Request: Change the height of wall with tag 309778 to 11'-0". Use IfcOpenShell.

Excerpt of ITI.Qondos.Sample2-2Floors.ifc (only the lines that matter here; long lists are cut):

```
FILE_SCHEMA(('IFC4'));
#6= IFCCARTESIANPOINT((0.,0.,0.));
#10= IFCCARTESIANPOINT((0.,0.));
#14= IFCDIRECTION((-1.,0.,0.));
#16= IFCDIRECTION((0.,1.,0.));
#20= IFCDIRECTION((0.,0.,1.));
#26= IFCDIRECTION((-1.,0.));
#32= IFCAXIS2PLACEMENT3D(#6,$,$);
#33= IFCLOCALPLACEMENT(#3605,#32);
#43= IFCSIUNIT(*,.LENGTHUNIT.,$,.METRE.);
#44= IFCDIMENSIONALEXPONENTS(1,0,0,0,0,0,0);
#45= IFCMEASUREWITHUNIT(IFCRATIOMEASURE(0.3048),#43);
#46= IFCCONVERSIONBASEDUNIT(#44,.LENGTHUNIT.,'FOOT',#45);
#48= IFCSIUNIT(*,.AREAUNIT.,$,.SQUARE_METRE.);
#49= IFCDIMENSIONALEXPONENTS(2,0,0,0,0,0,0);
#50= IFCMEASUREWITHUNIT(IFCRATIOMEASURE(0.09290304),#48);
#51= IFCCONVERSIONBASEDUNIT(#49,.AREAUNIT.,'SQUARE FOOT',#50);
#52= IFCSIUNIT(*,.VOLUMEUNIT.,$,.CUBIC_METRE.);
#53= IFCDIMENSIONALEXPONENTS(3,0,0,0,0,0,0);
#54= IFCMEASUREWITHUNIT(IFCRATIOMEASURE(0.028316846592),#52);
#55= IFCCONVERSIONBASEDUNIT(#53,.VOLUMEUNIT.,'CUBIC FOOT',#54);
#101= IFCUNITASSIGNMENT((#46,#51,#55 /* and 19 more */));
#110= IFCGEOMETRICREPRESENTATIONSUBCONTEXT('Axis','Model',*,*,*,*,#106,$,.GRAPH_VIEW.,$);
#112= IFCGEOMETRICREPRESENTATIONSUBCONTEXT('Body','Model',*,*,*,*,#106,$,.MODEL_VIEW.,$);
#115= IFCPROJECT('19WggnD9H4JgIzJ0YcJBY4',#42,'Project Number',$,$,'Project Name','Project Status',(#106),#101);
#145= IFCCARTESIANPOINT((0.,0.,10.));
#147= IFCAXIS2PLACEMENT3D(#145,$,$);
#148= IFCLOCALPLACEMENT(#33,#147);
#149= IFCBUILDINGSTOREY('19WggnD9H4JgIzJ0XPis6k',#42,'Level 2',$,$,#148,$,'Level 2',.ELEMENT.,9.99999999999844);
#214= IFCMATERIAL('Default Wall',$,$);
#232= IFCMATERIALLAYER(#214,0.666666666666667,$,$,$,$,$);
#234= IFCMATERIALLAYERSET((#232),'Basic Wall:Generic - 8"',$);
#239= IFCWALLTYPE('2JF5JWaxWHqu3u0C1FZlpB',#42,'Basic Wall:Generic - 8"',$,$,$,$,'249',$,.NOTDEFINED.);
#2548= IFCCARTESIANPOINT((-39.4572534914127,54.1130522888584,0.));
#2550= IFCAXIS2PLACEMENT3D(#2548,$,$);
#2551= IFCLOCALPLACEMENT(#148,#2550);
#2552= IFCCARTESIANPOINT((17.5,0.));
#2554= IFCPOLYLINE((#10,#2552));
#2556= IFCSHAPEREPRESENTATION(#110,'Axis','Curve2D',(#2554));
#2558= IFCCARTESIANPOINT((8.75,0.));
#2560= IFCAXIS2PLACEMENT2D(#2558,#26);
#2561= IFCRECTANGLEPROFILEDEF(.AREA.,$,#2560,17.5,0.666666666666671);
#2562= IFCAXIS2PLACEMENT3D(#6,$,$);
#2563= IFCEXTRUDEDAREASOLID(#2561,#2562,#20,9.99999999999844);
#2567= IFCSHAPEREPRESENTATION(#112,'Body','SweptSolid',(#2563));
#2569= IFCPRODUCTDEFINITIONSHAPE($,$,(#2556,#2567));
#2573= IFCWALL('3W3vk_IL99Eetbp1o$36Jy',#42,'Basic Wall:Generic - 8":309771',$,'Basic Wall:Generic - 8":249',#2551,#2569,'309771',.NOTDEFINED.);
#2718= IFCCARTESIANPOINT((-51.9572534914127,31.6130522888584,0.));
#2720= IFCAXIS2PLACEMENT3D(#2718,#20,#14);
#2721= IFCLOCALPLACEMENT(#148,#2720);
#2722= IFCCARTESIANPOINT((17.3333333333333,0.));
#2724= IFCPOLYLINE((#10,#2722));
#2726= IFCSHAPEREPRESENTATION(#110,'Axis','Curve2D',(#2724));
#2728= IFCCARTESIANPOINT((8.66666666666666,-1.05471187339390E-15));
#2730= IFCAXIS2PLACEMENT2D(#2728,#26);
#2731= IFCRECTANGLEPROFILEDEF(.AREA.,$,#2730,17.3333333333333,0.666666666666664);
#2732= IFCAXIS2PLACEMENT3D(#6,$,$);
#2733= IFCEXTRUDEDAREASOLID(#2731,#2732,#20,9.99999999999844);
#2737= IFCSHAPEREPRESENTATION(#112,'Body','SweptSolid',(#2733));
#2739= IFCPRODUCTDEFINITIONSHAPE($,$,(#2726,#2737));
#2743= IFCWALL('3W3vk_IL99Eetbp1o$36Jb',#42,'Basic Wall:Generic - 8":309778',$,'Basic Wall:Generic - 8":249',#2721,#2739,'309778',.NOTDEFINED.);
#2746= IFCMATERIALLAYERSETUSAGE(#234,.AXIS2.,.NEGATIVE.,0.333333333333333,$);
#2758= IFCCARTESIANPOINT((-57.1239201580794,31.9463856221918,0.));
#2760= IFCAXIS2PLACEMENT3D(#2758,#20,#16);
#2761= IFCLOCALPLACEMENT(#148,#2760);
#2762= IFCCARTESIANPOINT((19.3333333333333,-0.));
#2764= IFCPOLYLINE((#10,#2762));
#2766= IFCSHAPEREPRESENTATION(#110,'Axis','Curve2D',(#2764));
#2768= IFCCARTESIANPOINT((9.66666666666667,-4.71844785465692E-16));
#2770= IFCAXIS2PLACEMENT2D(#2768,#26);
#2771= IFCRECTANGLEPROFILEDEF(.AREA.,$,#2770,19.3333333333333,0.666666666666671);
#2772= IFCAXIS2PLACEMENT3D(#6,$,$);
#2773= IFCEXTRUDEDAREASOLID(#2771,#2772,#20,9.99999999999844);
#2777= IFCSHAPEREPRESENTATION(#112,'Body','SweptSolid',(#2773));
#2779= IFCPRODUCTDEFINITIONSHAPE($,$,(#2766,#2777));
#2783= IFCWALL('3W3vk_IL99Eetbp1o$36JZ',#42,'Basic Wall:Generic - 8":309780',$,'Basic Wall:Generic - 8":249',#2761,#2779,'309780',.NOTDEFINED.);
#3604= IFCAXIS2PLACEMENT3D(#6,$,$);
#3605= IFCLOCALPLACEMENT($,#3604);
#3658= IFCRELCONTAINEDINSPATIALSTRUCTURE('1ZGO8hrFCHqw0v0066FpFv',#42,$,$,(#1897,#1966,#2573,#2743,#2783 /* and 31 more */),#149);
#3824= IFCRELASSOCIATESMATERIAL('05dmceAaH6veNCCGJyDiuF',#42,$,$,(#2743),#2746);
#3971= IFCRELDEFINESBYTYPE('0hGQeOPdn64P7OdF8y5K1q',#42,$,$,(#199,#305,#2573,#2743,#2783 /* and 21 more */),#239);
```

```python
import ifcopenshell
import ifcopenshell.geom
import ifcopenshell.util.representation
import ifcopenshell.util.shape
import ifcopenshell.util.unit

model = ifcopenshell.open("ITI.Qondos.Sample2-2Floors.ifc")
unit_scale = ifcopenshell.util.unit.calculate_unit_scale(model)
settings = ifcopenshell.geom.settings()


def volume(element):
    """Net volume in cubic metres, openings subtracted."""
    shape = ifcopenshell.geom.create_shape(settings, element)
    return ifcopenshell.util.shape.get_volume(shape.geometry)


wall = model.by_guid("3W3vk_IL99Eetbp1o$36Jb")
before = volume(wall)

body = ifcopenshell.util.representation.get_representation(wall, "Model", "Body")
solid = body.Items[0]
old_height = solid.Depth
solid.Depth = 132 * 0.0254 / unit_scale
after = volume(wall)

print(f"height {old_height:g} -> {solid.Depth:g}, volume {before:.3f} -> {after:.3f} m3")

model.write("ITI.Qondos.Sample2-2Floors_updated.ifc")
```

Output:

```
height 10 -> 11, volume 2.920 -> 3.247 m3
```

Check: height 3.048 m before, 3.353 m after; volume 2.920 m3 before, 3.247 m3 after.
